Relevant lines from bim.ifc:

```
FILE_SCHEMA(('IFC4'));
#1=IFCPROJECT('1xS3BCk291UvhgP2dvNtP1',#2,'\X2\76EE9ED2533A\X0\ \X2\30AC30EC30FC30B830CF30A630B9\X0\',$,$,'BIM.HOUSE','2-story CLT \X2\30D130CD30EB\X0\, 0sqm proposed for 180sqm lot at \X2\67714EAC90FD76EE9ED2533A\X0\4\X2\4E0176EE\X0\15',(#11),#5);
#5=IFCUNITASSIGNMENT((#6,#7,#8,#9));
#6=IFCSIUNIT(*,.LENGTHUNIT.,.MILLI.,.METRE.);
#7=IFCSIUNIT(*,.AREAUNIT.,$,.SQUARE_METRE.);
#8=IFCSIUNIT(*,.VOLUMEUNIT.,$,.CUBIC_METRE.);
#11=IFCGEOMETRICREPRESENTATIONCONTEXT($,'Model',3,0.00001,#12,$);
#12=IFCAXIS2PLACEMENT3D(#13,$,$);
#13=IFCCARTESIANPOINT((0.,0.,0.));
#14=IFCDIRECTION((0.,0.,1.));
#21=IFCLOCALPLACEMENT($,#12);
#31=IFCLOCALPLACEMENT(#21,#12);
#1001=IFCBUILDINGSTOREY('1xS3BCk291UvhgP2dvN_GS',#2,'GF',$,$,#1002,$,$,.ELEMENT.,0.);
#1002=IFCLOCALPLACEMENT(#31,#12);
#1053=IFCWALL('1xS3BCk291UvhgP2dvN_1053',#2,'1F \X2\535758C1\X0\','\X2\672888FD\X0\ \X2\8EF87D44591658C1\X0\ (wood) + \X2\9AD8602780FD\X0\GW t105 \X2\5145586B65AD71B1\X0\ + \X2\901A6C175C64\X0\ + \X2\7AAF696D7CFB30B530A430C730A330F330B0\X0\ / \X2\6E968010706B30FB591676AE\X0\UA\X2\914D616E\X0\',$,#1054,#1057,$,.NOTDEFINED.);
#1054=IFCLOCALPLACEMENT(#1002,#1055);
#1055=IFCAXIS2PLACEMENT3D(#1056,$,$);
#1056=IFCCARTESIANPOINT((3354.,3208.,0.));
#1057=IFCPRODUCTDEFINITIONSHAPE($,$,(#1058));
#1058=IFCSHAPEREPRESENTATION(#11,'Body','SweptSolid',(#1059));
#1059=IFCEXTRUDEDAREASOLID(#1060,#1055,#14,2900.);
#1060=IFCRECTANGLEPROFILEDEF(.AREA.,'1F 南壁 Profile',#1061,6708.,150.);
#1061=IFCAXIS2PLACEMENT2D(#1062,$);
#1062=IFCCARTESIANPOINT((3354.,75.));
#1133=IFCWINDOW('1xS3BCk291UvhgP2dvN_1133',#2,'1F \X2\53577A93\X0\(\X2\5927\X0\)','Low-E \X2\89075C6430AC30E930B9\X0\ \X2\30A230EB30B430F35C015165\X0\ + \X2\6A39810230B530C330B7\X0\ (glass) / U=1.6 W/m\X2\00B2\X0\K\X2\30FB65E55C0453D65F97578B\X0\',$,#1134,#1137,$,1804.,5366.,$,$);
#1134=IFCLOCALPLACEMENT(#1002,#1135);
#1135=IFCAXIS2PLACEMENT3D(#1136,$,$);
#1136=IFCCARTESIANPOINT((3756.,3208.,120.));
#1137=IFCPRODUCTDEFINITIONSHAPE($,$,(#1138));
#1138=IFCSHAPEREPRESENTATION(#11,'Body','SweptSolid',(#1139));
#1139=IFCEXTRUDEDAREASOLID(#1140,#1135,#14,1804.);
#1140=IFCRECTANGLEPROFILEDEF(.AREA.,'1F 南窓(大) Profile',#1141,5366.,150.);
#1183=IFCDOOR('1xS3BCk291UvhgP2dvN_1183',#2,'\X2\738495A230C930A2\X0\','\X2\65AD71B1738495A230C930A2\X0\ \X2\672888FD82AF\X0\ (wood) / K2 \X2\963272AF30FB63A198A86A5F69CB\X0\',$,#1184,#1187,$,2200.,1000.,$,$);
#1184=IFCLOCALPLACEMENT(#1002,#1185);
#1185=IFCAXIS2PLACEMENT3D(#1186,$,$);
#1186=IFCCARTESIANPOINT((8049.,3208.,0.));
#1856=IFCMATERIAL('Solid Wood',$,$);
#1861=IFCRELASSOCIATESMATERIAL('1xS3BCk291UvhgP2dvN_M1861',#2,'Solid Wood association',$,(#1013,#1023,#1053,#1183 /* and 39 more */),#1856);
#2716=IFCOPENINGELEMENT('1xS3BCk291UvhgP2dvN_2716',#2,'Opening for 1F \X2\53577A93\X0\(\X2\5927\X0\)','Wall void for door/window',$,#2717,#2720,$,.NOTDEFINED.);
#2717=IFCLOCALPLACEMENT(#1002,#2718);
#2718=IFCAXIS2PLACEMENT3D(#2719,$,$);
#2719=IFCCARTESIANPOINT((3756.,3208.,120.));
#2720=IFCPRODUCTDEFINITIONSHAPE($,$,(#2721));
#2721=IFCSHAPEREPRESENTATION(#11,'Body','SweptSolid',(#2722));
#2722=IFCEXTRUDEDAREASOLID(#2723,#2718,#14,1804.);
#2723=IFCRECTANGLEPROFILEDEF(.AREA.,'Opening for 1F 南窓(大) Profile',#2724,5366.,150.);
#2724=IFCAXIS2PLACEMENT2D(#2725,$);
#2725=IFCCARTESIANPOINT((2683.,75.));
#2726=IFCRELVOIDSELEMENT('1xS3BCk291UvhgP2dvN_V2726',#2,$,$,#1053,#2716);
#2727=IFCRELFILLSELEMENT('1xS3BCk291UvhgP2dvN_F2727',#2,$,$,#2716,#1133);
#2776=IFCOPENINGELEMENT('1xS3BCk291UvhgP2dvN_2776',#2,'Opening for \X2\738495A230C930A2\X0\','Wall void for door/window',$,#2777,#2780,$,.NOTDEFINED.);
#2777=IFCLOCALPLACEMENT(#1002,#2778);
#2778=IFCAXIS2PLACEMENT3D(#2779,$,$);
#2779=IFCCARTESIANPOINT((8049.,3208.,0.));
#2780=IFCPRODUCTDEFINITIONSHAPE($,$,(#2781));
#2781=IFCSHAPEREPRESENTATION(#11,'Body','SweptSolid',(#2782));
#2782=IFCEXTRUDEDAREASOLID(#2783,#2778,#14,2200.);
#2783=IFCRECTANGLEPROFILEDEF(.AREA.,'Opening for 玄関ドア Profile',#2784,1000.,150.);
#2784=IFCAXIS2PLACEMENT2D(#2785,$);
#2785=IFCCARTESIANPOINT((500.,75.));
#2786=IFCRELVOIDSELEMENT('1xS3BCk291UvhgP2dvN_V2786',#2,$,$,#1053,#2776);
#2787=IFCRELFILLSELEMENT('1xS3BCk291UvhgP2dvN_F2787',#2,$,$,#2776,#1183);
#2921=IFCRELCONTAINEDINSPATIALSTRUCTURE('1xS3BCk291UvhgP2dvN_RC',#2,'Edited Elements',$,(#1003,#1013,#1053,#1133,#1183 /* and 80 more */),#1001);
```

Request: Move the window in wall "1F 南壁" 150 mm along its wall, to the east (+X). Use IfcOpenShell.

```python
import ifcopenshell
import ifcopenshell.api.geometry
import ifcopenshell.util.placement
import ifcopenshell.util.unit

model = ifcopenshell.open("bim.ifc")
unit_scale = ifcopenshell.util.unit.calculate_unit_scale(model)

window = model.by_id(1133)
opening = window.FillsVoids[0].RelatingOpeningElement
wall = opening.VoidsElements[0].RelatingBuildingElement

wall_matrix = ifcopenshell.util.placement.get_local_placement(wall.ObjectPlacement)
shift = wall_matrix[:3, 0] * 0.15 / unit_scale
before = ifcopenshell.util.placement.get_local_placement(window.ObjectPlacement)[:3, 3].copy()

# The window is not placed relative to its opening, so move both.
for product in (opening, window):
    matrix = ifcopenshell.util.placement.get_local_placement(product.ObjectPlacement)
    matrix[:3, 3] += shift
    ifcopenshell.api.geometry.edit_object_placement(model, product=product, matrix=matrix, is_si=False)

after = ifcopenshell.util.placement.get_local_placement(window.ObjectPlacement)[:3, 3]
print("window moved by", (after - before).round(3) + 0.0)

model.write("bim_v2.ifc")
```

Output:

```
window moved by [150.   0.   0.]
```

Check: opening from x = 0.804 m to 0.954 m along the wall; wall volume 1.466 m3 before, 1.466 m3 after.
